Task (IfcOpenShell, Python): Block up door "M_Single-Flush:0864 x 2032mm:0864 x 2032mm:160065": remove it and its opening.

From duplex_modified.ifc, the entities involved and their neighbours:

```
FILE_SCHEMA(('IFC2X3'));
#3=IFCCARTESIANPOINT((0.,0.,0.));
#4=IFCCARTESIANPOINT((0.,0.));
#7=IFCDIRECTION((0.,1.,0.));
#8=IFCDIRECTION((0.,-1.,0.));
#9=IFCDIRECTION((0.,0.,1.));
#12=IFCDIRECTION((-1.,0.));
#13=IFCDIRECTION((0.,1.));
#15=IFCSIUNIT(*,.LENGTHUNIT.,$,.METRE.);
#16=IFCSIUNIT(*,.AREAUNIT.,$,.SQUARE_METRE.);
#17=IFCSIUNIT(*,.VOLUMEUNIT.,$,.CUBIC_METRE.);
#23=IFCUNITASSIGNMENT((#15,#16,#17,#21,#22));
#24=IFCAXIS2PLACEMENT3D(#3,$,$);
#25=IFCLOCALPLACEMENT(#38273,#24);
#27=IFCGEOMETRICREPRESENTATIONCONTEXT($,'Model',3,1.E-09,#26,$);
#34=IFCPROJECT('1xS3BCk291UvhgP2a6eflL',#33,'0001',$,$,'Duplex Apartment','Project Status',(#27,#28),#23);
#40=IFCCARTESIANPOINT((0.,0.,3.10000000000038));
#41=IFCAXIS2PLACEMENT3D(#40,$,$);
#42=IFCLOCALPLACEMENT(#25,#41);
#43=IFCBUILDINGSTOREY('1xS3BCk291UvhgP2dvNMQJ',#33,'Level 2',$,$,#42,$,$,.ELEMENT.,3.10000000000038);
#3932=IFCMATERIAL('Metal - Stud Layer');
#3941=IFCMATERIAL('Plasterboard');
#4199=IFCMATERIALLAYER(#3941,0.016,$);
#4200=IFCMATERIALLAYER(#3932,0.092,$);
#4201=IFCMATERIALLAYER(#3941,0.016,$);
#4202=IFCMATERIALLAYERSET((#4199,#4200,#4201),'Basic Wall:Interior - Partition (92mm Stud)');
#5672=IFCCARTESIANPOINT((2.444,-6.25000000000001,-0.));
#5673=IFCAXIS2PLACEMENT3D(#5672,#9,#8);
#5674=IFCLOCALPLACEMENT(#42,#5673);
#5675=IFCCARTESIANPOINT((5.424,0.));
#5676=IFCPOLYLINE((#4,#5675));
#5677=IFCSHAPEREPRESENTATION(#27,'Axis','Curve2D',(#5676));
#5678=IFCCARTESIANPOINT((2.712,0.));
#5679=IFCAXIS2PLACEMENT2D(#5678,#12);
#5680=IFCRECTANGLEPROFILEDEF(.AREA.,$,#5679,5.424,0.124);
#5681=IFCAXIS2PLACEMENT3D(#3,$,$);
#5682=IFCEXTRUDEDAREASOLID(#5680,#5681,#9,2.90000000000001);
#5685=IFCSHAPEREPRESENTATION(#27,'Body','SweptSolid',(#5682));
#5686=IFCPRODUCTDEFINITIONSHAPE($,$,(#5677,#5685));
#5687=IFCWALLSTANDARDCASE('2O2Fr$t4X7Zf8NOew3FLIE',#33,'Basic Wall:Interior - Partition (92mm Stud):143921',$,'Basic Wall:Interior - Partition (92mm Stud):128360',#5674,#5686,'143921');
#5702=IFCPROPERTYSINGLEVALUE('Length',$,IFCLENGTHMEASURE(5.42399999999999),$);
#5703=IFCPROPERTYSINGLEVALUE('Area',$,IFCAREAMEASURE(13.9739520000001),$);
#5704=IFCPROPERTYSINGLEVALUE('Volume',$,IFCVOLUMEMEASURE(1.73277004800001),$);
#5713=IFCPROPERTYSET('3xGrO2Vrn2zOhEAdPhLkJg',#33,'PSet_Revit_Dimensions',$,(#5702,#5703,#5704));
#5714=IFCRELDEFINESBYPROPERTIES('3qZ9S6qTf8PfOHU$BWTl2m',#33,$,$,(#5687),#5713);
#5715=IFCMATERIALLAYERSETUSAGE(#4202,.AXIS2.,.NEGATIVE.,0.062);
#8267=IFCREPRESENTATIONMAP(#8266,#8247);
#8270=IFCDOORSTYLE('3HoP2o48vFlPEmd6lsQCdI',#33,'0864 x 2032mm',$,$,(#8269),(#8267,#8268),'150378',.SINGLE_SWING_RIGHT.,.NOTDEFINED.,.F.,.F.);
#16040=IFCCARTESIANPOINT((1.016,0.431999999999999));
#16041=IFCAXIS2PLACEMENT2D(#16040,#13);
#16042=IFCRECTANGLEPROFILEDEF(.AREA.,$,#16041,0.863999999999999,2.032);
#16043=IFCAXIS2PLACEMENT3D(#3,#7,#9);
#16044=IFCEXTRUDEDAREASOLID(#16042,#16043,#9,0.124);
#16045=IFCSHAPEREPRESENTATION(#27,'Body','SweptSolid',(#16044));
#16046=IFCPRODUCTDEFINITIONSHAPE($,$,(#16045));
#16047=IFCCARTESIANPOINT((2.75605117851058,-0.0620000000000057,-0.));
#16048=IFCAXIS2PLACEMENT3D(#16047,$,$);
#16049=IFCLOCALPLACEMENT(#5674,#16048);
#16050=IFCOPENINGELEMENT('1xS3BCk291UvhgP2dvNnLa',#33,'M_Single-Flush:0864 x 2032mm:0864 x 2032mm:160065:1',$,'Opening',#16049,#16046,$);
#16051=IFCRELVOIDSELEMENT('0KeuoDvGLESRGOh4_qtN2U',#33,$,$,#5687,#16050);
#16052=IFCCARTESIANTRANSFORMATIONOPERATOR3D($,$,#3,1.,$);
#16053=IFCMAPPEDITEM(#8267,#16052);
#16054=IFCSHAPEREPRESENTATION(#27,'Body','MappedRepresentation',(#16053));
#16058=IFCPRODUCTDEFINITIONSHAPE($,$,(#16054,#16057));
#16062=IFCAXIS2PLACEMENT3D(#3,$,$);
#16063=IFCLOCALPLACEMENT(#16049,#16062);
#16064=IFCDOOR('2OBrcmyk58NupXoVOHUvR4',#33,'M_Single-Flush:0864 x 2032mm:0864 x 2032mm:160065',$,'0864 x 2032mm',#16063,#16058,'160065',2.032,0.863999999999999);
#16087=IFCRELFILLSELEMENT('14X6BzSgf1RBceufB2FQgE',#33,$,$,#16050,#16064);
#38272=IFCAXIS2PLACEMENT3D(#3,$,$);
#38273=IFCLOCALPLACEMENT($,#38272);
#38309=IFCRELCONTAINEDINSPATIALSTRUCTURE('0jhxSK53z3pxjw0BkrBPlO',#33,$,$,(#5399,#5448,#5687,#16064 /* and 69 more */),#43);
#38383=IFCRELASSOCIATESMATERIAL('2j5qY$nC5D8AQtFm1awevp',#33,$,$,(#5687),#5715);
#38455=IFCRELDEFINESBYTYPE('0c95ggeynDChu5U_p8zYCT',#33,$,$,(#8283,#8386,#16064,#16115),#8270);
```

```python
import ifcopenshell
import ifcopenshell.api.feature
import ifcopenshell.api.pset
import ifcopenshell.api.root
import ifcopenshell.geom
import ifcopenshell.util.element
import ifcopenshell.util.shape
import ifcopenshell.util.unit

model = ifcopenshell.open("duplex_modified.ifc")
area_scale = ifcopenshell.util.unit.calculate_unit_scale(model, "AREAUNIT")
volume_scale = ifcopenshell.util.unit.calculate_unit_scale(model, "VOLUMEUNIT")
settings = ifcopenshell.geom.settings()


def volume(element):
    """Net volume in cubic metres, openings subtracted."""
    shape = ifcopenshell.geom.create_shape(settings, element)
    return ifcopenshell.util.shape.get_volume(shape.geometry)


door = model.by_guid("2OBrcmyk58NupXoVOHUvR4")
opening = door.FillsVoids[0].RelatingOpeningElement
wall = opening.VoidsElements[0].RelatingBuildingElement
before = volume(wall)

ifcopenshell.api.root.remove_product(model, product=door)
ifcopenshell.api.feature.remove_feature(model, feature=opening)

after = volume(wall)
thickness = 0.124  # wall thickness in metres

# Update the wall's stored quantities.
pset = model.by_id(ifcopenshell.util.element.get_pset(wall, "PSet_Revit_Dimensions", should_inherit=False)["id"])
ifcopenshell.api.pset.edit_pset(model, pset=pset, properties={
    "Area": model.create_entity("IfcAreaMeasure", after / thickness / area_scale),
    "Volume": model.create_entity("IfcVolumeMeasure", after / volume_scale),
})

print(f"wall volume {before:.3f} -> {after:.3f} m3")

model.write("duplex_modified-out.ifc")
```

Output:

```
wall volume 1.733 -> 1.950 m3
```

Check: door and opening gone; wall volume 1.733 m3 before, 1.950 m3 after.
